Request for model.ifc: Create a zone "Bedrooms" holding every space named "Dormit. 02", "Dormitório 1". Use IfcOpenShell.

First a look at what the model holds.

```python
import ifcopenshell

model = ifcopenshell.open("model.ifc")
print(model.schema)
seen = {}
for space in model.by_type("IfcSpace"):
    seen[space.LongName] = seen.get(space.LongName, 0) + 1
for name, count in sorted(seen.items(), key=str):
    print(count, "x", name)
print("zones:", [z.Name for z in model.by_type("IfcZone")][:20])
```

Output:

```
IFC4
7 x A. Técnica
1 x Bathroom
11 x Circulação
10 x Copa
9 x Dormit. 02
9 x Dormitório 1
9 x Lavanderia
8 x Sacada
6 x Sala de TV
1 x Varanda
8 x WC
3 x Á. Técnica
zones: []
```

```python
import ifcopenshell
import ifcopenshell.api.group
import ifcopenshell.api.root

model = ifcopenshell.open("model.ifc")

names = {"Dormit. 02", "Dormitório 1"}
spaces = [s for s in model.by_type("IfcSpace") if s.LongName in names]

zone = ifcopenshell.api.root.create_entity(model, ifc_class="IfcZone", name="Bedrooms")
ifcopenshell.api.group.assign_group(model, products=spaces, group=zone)
print(len(spaces), "spaces in", zone.Name)

model.write("model_edited.ifc")
```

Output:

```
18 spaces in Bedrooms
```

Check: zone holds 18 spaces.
